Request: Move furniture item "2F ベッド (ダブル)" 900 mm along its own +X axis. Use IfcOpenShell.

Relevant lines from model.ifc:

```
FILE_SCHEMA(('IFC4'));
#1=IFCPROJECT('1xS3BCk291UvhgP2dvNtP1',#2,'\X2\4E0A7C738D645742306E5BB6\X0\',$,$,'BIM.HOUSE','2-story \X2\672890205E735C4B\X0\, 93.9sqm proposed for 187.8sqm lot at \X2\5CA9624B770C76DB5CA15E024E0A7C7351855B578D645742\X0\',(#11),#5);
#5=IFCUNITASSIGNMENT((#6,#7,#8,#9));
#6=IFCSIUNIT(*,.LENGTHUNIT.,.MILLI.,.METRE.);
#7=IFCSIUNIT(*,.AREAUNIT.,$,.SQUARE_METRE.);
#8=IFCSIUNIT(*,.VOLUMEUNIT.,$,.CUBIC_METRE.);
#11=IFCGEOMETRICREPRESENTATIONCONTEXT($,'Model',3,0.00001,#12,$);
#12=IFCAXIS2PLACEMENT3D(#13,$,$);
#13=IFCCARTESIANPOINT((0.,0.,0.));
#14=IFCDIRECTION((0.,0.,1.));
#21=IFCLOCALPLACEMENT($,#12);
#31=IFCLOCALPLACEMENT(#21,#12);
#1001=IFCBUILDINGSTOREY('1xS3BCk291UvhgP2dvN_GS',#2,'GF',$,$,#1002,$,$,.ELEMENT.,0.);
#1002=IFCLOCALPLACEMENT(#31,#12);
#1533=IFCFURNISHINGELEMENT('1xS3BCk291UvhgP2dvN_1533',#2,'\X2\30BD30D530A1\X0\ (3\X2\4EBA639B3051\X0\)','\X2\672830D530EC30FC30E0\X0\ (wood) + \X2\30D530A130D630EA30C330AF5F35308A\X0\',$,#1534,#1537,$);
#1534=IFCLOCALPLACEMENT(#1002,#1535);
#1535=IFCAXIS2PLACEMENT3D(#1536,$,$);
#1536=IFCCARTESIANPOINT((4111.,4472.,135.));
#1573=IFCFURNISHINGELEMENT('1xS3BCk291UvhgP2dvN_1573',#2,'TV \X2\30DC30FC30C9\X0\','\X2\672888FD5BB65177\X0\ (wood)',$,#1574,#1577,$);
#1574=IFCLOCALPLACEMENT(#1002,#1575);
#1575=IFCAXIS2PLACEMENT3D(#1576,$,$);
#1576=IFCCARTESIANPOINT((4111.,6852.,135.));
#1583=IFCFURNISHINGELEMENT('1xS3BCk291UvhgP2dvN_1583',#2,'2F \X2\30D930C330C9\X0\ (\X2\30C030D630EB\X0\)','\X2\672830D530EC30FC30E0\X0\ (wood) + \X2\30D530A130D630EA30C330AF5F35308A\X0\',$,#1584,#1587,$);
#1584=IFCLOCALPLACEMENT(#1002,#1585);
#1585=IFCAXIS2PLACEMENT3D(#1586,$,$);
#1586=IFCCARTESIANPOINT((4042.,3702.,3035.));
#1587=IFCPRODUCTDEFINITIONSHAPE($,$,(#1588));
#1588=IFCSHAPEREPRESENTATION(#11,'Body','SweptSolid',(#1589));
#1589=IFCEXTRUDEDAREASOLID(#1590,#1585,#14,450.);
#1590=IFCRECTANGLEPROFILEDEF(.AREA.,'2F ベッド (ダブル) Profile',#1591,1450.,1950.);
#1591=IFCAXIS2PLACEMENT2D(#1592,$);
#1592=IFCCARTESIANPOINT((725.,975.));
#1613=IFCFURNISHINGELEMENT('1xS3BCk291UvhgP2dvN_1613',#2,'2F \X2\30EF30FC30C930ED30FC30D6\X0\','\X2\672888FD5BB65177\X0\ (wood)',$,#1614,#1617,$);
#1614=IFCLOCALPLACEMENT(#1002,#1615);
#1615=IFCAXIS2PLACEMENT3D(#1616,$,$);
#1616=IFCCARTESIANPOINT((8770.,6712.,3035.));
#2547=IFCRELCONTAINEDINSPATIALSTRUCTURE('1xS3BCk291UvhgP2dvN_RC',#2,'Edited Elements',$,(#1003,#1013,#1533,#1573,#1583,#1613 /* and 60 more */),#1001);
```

```python
import ifcopenshell
import ifcopenshell.api.geometry
import ifcopenshell.util.placement

model = ifcopenshell.open("model.ifc")

item = model.by_guid("1xS3BCk291UvhgP2dvN_1583")
matrix = ifcopenshell.util.placement.get_local_placement(item.ObjectPlacement)
matrix[:3, 3] += matrix[:3, 0] * 900.0
ifcopenshell.api.geometry.edit_object_placement(model, product=item, matrix=matrix, is_si=False)

print(ifcopenshell.util.placement.get_local_placement(item.ObjectPlacement).round(3) + 0.0)

model.write("model_updated.ifc")
```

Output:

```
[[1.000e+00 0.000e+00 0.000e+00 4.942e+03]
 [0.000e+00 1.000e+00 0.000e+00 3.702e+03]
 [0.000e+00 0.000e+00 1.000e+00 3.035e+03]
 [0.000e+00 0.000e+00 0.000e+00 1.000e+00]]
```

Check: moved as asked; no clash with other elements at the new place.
